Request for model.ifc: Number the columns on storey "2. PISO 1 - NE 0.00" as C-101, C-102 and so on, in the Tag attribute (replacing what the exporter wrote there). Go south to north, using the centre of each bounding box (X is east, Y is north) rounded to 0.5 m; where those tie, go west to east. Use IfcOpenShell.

First a look at what the model holds.

```python
import ifcopenshell
import ifcopenshell.util.element
import ifcopenshell.util.placement

model = ifcopenshell.open("model.ifc")
print(model.schema)
storey = next(s for s in model.by_type("IfcBuildingStorey") if s.Name == "2. PISO 1 - NE 0.00")
columns = [e for e in ifcopenshell.util.element.get_decomposition(storey) if e.is_a("IfcColumn")]
for e in sorted(columns, key=lambda e: e.id()):
    origin = ifcopenshell.util.placement.get_local_placement(e.ObjectPlacement)[:3, 3]
    print(e.id(), e.Tag, e.Name, origin.round(2) + 0.0, sep=" | ")
```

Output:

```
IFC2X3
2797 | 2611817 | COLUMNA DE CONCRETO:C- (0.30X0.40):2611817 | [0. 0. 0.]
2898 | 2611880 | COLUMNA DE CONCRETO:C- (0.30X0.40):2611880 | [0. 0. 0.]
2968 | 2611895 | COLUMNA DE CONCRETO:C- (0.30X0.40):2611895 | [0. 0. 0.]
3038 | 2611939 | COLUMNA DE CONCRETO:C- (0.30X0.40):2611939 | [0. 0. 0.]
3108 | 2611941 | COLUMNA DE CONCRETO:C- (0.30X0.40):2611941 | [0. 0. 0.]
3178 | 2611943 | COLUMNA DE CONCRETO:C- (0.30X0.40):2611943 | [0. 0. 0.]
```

```python
import ifcopenshell
import ifcopenshell.geom
import ifcopenshell.util.element
import ifcopenshell.util.shape

model = ifcopenshell.open("model.ifc")
settings = ifcopenshell.geom.settings()
settings.set("use-world-coords", True)


def centre(element):
    shape = ifcopenshell.geom.create_shape(settings, element)
    return ifcopenshell.util.shape.get_bbox_centroid(shape.geometry)


storey = next(s for s in model.by_type("IfcBuildingStorey") if s.Name == "2. PISO 1 - NE 0.00")
columns = [e for e in ifcopenshell.util.element.get_decomposition(storey) if e.is_a("IfcColumn")]

# Insertion points can sit at a corner or the storey origin, so sort by the geometry (in metres).
centres = {e: centre(e) for e in columns}
columns.sort(key=lambda e: (round(centres[e][1] / 0.5), centres[e][0]))

for i, e in enumerate(columns, start=1):
    number = f"C-1{i:02d}"
    e.Tag = number
    print(e.id(), number)

model.write("model_edited.ifc")
```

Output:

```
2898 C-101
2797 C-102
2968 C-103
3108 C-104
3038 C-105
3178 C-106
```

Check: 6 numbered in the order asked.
